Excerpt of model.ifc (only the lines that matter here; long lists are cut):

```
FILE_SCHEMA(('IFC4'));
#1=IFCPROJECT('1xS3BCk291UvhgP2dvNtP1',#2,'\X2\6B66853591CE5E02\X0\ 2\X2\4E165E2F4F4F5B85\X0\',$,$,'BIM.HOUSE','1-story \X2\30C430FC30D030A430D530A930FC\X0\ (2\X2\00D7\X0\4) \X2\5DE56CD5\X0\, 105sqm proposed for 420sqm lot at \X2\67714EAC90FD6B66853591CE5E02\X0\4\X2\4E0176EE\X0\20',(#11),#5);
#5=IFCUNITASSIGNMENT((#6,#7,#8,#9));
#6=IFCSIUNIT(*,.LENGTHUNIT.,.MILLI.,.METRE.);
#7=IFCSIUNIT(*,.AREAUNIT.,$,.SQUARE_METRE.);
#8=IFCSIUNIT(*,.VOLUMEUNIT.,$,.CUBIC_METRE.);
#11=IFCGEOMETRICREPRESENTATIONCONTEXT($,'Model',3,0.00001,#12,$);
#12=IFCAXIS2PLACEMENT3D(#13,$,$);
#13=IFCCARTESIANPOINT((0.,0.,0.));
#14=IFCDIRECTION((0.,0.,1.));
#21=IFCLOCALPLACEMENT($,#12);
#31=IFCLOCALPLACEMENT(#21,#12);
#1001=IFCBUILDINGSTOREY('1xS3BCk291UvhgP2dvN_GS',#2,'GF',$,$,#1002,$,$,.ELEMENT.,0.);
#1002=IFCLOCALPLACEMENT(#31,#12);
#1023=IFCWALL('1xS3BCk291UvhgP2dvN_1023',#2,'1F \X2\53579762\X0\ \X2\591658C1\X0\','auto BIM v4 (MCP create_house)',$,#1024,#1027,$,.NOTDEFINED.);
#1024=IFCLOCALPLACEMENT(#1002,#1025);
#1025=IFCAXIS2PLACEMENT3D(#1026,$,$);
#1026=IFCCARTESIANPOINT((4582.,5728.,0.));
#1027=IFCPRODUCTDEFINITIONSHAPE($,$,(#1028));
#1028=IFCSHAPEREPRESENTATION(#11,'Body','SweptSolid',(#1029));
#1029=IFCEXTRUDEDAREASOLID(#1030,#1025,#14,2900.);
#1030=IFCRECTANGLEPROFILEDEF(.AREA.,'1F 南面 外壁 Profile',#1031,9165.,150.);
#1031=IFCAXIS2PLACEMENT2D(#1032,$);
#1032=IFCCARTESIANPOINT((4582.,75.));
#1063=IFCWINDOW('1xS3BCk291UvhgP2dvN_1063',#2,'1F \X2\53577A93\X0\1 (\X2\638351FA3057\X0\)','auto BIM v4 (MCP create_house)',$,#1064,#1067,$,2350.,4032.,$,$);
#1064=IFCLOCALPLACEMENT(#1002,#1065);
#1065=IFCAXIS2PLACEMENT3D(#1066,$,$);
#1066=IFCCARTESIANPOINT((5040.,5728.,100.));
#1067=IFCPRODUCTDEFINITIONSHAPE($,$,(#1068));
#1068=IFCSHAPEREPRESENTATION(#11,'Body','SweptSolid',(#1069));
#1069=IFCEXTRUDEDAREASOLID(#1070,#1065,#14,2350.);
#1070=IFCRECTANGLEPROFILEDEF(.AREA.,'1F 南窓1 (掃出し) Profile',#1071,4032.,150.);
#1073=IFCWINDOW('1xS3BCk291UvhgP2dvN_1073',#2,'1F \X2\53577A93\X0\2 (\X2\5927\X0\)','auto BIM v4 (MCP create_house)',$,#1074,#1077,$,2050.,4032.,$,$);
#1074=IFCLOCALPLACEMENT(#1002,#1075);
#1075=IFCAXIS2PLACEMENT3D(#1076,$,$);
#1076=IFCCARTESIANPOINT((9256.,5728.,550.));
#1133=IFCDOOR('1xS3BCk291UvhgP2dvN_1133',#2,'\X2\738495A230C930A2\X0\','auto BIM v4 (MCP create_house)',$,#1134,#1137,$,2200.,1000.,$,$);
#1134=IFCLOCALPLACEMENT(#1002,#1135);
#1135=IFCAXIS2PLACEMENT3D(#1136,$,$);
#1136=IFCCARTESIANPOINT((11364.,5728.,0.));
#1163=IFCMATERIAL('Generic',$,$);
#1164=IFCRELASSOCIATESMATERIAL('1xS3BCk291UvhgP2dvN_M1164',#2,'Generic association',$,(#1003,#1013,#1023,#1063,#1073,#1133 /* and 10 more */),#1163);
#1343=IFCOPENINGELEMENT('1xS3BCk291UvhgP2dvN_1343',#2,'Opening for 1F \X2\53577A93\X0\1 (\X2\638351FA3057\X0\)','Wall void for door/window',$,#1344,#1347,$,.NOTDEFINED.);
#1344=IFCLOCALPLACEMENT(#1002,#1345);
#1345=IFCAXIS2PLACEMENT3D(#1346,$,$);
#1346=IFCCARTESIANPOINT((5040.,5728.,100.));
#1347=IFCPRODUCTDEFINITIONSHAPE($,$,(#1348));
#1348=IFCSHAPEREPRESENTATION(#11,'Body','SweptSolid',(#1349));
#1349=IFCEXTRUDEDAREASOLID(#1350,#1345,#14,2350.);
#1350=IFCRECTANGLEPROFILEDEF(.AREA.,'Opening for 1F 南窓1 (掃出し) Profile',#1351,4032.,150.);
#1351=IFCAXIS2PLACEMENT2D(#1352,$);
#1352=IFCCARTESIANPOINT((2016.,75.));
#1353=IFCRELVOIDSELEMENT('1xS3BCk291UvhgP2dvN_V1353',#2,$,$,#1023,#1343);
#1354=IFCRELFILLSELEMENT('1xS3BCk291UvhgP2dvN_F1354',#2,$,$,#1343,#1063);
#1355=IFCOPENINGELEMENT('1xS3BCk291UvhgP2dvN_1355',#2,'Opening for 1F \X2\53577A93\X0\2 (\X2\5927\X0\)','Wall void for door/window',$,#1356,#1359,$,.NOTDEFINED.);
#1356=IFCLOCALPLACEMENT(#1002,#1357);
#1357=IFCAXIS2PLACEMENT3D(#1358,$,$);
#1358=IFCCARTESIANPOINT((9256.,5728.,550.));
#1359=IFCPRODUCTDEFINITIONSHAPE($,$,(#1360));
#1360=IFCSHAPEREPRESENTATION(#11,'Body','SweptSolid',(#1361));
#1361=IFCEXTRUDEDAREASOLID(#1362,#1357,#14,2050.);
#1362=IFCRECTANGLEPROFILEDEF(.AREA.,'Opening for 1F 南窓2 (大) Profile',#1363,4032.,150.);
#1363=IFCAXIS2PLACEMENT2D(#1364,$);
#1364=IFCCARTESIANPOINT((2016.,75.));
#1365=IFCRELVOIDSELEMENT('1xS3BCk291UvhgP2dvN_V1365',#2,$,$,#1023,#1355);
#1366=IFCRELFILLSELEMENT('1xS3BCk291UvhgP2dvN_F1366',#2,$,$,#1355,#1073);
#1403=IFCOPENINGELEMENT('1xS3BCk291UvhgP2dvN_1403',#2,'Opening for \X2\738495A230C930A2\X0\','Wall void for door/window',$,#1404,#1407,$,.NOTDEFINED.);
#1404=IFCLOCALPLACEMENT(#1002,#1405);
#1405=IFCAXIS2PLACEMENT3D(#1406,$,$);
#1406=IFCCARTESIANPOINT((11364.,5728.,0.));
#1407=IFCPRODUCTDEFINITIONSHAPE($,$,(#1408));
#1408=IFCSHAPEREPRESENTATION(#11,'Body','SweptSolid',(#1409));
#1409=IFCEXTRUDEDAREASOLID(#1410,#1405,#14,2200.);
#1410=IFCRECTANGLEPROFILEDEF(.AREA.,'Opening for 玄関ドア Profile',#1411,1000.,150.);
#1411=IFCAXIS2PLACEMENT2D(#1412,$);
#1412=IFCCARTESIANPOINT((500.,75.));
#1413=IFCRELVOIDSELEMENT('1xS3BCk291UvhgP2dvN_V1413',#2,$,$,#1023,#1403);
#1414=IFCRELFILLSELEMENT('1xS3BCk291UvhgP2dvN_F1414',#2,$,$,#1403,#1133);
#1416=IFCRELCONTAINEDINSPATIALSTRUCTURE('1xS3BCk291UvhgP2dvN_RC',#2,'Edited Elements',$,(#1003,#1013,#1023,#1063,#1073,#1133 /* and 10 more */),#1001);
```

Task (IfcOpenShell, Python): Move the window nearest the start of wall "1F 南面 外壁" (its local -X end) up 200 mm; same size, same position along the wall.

```python
import numpy as np
import ifcopenshell
import ifcopenshell.api.geometry
import ifcopenshell.util.placement
import ifcopenshell.util.unit

model = ifcopenshell.open("model.ifc")
unit_scale = ifcopenshell.util.unit.calculate_unit_scale(model)

window = model.by_id(1063)
opening = window.FillsVoids[0].RelatingOpeningElement
dz = 0.2 / unit_scale

shift = np.array([0.0, 0.0, dz])
# The window is not placed relative to its opening, so move both.
for product in (opening, window):
    matrix = ifcopenshell.util.placement.get_local_placement(product.ObjectPlacement)
    matrix[:3, 3] += shift
    ifcopenshell.api.geometry.edit_object_placement(model, product=product, matrix=matrix, is_si=False)

print(f"moved by {dz * unit_scale:+.3f} m")

model.write("model-out.ifc")
```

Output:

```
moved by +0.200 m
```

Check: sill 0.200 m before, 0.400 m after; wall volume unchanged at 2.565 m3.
